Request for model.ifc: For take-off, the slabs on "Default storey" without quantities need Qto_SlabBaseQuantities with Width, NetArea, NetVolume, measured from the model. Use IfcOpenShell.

First a look at what the model holds.

```python
import ifcopenshell
import ifcopenshell.util.element
import ifcopenshell.util.unit

model = ifcopenshell.open("model.ifc")
print(model.schema)
for unit_type in ("LENGTHUNIT", "AREAUNIT", "VOLUMEUNIT"):
    print(unit_type, ifcopenshell.util.unit.calculate_unit_scale(model, unit_type))
storey = next(s for s in model.by_type("IfcBuildingStorey") if s.Name == "Default storey")
slabs = [e for e in ifcopenshell.util.element.get_decomposition(storey) if e.is_a("IfcSlab")]
for e in sorted(slabs, key=lambda e: e.id()):
    print(e.id(), e.is_a(), e.Name, list(ifcopenshell.util.element.get_psets(e, qtos_only=True)), sep=" | ")
```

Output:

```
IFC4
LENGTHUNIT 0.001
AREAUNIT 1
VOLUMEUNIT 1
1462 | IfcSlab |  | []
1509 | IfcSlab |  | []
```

```python
import ifcopenshell
import ifcopenshell.api.pset
import ifcopenshell.geom
import ifcopenshell.util.element
import ifcopenshell.util.shape
import ifcopenshell.util.unit

model = ifcopenshell.open("model.ifc")
unit_scale = ifcopenshell.util.unit.calculate_unit_scale(model)
area_scale = ifcopenshell.util.unit.calculate_unit_scale(model, "AREAUNIT")
volume_scale = ifcopenshell.util.unit.calculate_unit_scale(model, "VOLUMEUNIT")
settings = ifcopenshell.geom.settings()

storey = next(s for s in model.by_type("IfcBuildingStorey") if s.Name == "Default storey")
slabs = [e for e in ifcopenshell.util.element.get_decomposition(storey) if e.is_a("IfcSlab")]

for e in sorted(slabs, key=lambda e: e.id()):
    if ifcopenshell.util.element.get_psets(e, qtos_only=True, should_inherit=False):
        continue
    # Geometry comes back in metres, in the element's own axes.
    shape = ifcopenshell.geom.create_shape(settings, e)
    values = {
        "Width": ifcopenshell.util.shape.get_z(shape.geometry) / unit_scale,
        "NetArea": ifcopenshell.util.shape.get_footprint_area(shape.geometry) / area_scale,
        "NetVolume": ifcopenshell.util.shape.get_volume(shape.geometry) / volume_scale,
    }
    qto = ifcopenshell.api.pset.add_qto(model, product=e, name="Qto_SlabBaseQuantities")
    ifcopenshell.api.pset.edit_qto(model, qto=qto, properties=values)
    print(e.id(), {k: round(v, 3) for k, v in values.items()})

model.write("model_rev.ifc")
```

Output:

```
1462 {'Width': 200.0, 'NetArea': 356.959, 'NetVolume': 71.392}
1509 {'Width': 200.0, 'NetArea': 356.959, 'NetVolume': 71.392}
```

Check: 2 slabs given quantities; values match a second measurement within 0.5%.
